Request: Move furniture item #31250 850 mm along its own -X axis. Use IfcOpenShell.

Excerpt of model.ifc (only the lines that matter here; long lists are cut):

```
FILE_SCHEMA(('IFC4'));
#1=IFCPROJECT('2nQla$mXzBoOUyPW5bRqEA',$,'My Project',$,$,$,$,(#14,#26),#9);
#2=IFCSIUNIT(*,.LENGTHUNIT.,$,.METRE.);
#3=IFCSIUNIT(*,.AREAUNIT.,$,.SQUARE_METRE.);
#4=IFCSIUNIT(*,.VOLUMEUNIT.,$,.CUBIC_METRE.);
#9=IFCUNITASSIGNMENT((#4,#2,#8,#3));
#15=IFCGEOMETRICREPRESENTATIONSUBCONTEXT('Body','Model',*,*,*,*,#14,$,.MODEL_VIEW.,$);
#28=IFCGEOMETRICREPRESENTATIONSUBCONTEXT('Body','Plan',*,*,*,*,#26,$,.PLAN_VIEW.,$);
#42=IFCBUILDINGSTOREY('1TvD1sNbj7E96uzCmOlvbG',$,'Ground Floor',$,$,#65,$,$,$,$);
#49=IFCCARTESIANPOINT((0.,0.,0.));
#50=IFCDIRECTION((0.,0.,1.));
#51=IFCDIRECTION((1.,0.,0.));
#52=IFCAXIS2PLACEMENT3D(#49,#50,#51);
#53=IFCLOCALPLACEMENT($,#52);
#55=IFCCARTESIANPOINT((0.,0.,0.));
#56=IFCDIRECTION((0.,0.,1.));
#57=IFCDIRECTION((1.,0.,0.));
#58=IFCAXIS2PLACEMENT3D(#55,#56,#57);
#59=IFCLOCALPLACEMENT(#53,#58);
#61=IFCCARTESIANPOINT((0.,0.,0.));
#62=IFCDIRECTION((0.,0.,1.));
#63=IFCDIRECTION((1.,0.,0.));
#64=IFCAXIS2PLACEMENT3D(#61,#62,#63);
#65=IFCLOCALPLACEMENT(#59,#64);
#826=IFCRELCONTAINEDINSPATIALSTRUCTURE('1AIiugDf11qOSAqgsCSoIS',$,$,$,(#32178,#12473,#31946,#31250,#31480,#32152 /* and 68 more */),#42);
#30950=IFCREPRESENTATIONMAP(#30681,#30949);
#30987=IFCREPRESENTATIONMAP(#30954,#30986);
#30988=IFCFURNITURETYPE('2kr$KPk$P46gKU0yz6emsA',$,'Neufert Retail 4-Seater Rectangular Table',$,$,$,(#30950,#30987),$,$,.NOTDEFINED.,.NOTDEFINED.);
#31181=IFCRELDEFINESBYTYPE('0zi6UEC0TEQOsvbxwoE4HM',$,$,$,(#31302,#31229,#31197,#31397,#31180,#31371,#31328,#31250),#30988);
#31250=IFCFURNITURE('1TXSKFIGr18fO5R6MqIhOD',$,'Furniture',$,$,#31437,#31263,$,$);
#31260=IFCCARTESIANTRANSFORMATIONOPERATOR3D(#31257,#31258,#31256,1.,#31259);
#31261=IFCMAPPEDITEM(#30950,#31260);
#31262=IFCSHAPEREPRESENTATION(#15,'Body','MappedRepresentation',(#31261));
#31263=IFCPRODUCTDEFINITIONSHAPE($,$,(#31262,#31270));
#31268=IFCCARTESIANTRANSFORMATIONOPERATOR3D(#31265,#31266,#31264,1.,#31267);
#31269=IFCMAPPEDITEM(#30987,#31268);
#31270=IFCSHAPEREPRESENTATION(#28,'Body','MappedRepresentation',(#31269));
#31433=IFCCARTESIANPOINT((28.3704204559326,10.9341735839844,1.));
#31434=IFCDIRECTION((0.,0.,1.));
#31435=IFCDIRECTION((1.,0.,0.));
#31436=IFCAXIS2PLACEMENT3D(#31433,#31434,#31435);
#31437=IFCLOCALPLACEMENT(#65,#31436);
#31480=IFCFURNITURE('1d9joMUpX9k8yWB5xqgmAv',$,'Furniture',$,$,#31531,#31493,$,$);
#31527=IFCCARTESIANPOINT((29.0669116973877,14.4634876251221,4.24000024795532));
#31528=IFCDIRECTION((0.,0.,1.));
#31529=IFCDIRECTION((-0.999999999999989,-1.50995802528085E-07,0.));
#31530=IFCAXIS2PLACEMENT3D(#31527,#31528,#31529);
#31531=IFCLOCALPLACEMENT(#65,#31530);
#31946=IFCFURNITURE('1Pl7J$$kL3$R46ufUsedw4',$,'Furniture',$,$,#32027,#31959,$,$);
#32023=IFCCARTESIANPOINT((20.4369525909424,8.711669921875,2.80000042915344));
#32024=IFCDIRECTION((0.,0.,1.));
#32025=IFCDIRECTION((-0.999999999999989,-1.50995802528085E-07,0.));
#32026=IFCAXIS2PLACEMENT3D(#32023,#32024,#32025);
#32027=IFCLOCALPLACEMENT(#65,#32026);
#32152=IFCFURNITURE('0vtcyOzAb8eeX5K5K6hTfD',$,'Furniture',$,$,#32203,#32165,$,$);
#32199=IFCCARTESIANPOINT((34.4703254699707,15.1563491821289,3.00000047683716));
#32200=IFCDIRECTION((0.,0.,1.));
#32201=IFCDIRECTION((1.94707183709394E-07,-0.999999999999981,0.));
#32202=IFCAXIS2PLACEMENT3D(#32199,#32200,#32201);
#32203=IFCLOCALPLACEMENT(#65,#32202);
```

```python
import ifcopenshell
import ifcopenshell.api.geometry
import ifcopenshell.util.placement

model = ifcopenshell.open("model.ifc")

item = model.by_guid("1TXSKFIGr18fO5R6MqIhOD")
matrix = ifcopenshell.util.placement.get_local_placement(item.ObjectPlacement)
matrix[:3, 3] -= matrix[:3, 0] * 0.85
ifcopenshell.api.geometry.edit_object_placement(model, product=item, matrix=matrix, is_si=False)

print(ifcopenshell.util.placement.get_local_placement(item.ObjectPlacement).round(3) + 0.0)

model.write("model_updated.ifc")
```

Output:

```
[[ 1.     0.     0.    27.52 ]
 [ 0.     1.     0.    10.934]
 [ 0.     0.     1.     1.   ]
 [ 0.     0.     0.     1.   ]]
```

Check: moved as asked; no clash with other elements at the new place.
